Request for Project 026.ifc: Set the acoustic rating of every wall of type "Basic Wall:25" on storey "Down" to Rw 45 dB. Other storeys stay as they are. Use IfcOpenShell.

First a look at what the model holds.

```python
import ifcopenshell
import ifcopenshell.util.element

model = ifcopenshell.open("Project 026.ifc")
print(model.schema)
storey = next(s for s in model.by_type("IfcBuildingStorey") if s.Name == "Down")
walls = [e for e in ifcopenshell.util.element.get_decomposition(storey) if e.is_a("IfcWall")]
seen = {}
for e in walls:
    element_type = ifcopenshell.util.element.get_type(e)
    key = (element_type.Name if element_type != e and element_type else None, ifcopenshell.util.element.get_pset(e, "Pset_WallCommon", "AcousticRating"))
    seen[key] = seen.get(key, 0) + 1
for (name, value), count in sorted(seen.items(), key=str):
    print(count, "x", name, "|", value)
```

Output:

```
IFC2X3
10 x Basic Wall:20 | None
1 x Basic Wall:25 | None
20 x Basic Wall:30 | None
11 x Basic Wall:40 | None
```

```python
import ifcopenshell
import ifcopenshell.api.pset
import ifcopenshell.util.element

model = ifcopenshell.open("Project 026.ifc")

storey = next(s for s in model.by_type("IfcBuildingStorey") if s.Name == "Down")
walls = [e for e in ifcopenshell.util.element.get_decomposition(storey) if e.is_a("IfcWall")]

count = 0
for e in walls:
    element_type = ifcopenshell.util.element.get_type(e)
    if element_type in (None, e) or element_type.Name != "Basic Wall:25":
        continue
    # add_pset returns the element's existing set when there is one.
    pset = ifcopenshell.api.pset.add_pset(model, product=e, name="Pset_WallCommon")
    ifcopenshell.api.pset.edit_pset(model, pset=pset, properties={"AcousticRating": "Rw 45 dB"})
    count += 1

print(count, "walls updated")

model.write("Project 026_v2.ifc")
```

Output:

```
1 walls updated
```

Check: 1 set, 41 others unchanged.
